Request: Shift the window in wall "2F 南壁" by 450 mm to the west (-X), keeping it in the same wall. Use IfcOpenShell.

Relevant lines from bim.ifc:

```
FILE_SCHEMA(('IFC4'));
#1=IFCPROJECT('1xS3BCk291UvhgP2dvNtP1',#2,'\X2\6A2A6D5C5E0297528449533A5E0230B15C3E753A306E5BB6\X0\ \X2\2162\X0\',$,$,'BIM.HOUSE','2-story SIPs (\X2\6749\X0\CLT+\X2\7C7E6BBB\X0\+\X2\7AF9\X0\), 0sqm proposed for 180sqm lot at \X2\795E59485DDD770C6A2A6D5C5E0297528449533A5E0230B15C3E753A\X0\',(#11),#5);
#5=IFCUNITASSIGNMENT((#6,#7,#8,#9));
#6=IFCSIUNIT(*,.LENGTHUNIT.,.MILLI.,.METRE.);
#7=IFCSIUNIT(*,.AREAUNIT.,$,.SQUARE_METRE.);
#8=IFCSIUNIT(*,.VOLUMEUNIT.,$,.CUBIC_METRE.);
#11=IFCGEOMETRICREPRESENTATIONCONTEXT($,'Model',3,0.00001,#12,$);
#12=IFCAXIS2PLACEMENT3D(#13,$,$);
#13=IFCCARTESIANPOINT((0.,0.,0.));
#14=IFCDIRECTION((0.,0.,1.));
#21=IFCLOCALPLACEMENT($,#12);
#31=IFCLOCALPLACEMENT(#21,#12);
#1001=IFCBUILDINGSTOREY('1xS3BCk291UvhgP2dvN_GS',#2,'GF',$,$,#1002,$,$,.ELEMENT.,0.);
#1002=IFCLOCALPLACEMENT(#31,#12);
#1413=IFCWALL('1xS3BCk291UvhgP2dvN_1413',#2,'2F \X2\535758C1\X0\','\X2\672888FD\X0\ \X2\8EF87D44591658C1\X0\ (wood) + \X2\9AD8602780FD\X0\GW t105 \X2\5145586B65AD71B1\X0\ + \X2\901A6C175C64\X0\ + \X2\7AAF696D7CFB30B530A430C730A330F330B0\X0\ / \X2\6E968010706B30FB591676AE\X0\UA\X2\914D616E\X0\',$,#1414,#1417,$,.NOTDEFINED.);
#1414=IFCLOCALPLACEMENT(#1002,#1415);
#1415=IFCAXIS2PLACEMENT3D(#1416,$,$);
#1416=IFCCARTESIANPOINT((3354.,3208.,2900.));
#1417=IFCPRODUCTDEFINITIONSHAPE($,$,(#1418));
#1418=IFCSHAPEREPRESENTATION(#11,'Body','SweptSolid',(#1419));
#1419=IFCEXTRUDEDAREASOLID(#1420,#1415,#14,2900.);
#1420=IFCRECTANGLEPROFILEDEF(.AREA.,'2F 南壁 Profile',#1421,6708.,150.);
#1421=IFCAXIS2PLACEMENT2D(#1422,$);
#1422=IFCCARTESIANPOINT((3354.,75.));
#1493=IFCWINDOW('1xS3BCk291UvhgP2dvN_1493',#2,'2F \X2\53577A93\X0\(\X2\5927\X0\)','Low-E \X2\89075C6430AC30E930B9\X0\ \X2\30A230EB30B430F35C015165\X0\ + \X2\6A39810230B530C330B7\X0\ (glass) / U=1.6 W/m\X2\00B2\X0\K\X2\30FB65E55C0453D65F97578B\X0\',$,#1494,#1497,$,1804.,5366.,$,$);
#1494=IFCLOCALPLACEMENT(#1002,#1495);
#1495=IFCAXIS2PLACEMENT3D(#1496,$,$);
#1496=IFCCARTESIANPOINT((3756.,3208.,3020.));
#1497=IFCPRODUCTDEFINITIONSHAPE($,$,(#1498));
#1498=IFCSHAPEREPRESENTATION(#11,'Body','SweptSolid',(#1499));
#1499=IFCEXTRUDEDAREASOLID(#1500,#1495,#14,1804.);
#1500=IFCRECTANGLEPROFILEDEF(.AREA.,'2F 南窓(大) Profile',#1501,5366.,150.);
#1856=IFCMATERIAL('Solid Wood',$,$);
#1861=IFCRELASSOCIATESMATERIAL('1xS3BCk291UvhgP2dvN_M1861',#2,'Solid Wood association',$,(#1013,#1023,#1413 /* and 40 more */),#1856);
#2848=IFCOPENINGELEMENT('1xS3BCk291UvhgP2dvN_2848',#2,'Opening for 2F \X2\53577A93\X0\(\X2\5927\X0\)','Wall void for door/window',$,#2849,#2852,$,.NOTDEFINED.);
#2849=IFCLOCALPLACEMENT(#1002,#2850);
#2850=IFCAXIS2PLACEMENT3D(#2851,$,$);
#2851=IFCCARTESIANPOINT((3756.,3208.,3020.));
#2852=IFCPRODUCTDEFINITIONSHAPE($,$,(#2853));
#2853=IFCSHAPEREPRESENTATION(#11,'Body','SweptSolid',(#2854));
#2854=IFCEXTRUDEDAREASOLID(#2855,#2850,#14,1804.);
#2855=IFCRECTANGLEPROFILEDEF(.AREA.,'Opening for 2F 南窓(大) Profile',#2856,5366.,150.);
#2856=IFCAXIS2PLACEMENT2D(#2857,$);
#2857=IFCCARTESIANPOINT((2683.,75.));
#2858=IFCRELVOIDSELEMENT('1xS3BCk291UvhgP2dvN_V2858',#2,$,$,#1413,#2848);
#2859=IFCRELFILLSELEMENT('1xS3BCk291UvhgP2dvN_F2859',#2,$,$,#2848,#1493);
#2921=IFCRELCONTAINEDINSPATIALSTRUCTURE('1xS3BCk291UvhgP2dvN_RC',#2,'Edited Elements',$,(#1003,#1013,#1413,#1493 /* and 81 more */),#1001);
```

```python
import ifcopenshell
import ifcopenshell.api.geometry
import ifcopenshell.util.placement

model = ifcopenshell.open("bim.ifc")

window = model.by_guid("1xS3BCk291UvhgP2dvN_1493")
opening = window.FillsVoids[0].RelatingOpeningElement
wall = opening.VoidsElements[0].RelatingBuildingElement

wall_matrix = ifcopenshell.util.placement.get_local_placement(wall.ObjectPlacement)
shift = wall_matrix[:3, 0] * -450.0
before = ifcopenshell.util.placement.get_local_placement(window.ObjectPlacement)[:3, 3].copy()

# The window is not placed relative to its opening, so move both.
for product in (opening, window):
    matrix = ifcopenshell.util.placement.get_local_placement(product.ObjectPlacement)
    matrix[:3, 3] += shift
    ifcopenshell.api.geometry.edit_object_placement(model, product=product, matrix=matrix, is_si=False)

after = ifcopenshell.util.placement.get_local_placement(window.ObjectPlacement)[:3, 3]
print("window moved by", (after - before).round(3) + 0.0)

model.write("bim-out.ifc")
```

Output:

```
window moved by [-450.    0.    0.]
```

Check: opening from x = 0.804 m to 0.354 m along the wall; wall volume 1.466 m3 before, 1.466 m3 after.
